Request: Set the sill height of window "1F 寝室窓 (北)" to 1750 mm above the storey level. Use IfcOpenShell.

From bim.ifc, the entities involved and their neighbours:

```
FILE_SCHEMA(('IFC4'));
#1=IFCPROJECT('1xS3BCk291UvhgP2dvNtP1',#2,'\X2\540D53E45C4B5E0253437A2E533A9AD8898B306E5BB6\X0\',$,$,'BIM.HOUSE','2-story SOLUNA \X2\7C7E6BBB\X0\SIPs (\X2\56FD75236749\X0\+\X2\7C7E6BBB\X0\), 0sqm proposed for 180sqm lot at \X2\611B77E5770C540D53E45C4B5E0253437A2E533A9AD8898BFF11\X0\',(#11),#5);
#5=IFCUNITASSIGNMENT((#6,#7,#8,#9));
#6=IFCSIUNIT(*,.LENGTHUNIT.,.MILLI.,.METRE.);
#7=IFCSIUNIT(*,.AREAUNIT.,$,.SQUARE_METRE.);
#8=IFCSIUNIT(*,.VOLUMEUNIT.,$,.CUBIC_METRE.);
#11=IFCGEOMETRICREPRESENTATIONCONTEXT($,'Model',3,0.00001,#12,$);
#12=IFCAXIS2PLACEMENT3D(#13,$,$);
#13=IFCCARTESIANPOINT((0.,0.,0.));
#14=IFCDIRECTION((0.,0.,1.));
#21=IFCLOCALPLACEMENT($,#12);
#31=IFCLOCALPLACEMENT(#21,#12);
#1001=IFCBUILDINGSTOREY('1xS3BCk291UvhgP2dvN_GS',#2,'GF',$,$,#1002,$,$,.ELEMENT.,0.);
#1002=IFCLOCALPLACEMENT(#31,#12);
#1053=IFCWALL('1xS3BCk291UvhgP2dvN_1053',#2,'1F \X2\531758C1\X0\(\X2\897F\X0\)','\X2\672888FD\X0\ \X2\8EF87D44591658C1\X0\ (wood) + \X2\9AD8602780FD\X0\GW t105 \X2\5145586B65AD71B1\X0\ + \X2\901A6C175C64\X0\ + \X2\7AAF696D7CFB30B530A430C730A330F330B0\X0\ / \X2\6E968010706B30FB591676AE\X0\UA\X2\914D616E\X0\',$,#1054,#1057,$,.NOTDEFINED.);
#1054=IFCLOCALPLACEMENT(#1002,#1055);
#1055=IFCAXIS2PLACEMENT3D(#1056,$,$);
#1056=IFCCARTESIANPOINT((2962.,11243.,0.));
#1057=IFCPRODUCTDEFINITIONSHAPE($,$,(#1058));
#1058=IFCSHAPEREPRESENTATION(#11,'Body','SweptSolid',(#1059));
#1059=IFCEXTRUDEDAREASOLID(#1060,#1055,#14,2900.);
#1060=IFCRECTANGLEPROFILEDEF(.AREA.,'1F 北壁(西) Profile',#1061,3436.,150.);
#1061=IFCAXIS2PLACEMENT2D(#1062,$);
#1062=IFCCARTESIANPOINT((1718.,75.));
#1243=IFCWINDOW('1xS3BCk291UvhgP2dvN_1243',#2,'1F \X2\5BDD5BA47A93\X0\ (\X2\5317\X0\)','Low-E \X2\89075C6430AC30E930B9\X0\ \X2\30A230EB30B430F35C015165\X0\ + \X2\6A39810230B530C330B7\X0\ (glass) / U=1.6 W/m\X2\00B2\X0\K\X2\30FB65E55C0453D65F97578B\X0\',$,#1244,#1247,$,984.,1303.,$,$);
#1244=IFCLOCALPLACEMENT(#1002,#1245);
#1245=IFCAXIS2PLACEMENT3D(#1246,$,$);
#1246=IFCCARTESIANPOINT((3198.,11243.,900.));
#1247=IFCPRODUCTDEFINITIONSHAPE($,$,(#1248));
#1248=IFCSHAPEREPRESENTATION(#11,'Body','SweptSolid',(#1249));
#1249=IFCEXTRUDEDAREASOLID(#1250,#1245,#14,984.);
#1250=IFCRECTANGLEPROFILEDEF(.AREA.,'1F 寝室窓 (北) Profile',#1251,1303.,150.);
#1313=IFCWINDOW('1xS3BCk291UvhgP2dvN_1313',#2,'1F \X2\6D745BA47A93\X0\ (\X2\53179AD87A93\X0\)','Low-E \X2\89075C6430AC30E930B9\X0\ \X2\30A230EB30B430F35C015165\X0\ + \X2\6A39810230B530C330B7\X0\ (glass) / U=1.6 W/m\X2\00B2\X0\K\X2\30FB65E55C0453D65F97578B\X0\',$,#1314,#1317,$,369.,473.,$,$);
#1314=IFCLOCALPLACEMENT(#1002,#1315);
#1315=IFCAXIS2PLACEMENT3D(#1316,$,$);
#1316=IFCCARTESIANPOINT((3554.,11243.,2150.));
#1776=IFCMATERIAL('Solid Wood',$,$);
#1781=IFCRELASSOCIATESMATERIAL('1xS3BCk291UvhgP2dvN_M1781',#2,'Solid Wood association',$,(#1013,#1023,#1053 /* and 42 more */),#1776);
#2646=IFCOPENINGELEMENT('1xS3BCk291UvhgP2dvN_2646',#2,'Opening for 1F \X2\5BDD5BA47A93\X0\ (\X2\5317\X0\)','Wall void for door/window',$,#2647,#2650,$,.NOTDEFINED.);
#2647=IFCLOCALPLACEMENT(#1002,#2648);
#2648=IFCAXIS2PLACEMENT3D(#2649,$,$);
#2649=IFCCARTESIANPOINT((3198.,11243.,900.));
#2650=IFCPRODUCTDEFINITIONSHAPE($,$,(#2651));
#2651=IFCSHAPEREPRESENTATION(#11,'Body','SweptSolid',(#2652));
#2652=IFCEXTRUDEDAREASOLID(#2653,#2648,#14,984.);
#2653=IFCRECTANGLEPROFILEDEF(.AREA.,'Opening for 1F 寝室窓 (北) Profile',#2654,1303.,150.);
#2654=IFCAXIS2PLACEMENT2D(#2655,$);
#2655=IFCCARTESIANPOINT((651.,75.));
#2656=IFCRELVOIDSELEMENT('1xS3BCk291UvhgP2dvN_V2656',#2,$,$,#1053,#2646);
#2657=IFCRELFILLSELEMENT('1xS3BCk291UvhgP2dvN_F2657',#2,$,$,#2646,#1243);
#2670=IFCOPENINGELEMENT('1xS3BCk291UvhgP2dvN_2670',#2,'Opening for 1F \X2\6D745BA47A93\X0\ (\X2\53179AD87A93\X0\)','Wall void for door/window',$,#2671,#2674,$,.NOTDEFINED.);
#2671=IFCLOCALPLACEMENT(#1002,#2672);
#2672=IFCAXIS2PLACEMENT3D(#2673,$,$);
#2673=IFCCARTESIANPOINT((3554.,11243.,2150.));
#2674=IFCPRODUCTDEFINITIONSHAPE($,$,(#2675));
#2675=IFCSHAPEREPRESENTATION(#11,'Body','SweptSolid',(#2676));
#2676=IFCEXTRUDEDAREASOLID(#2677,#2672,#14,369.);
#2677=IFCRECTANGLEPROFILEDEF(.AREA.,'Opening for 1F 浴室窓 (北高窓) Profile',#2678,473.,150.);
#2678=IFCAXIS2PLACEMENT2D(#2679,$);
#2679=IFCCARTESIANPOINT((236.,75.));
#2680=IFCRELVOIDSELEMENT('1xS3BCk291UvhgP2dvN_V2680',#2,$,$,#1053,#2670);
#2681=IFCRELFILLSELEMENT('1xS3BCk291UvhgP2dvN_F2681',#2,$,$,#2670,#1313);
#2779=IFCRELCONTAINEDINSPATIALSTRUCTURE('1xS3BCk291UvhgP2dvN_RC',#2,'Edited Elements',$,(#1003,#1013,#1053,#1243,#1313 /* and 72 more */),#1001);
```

```python
import numpy as np
import ifcopenshell
import ifcopenshell.api.geometry
import ifcopenshell.geom
import ifcopenshell.util.element
import ifcopenshell.util.placement
import ifcopenshell.util.shape
import ifcopenshell.util.unit

model = ifcopenshell.open("bim.ifc")
unit_scale = ifcopenshell.util.unit.calculate_unit_scale(model)

window = model.by_guid("1xS3BCk291UvhgP2dvN_1243")
opening = window.FillsVoids[0].RelatingOpeningElement
storey = ifcopenshell.util.element.get_container(window, ifc_class="IfcBuildingStorey")
level = ifcopenshell.util.placement.get_local_placement(storey.ObjectPlacement)[2, 3]

# The opening's origin need not be at the sill, so measure its lowest point.
shape = ifcopenshell.geom.create_shape(ifcopenshell.geom.settings(), opening)
bottom = ifcopenshell.util.shape.get_shape_bottom_elevation(shape, shape.geometry) / unit_scale
dz = level + 1.75 / unit_scale - bottom

shift = np.array([0.0, 0.0, dz])
# The window is not placed relative to its opening, so move both.
for product in (opening, window):
    matrix = ifcopenshell.util.placement.get_local_placement(product.ObjectPlacement)
    matrix[:3, 3] += shift
    ifcopenshell.api.geometry.edit_object_placement(model, product=product, matrix=matrix, is_si=False)

print(f"moved by {dz * unit_scale:+.3f} m")

model.write("bim_v2.ifc")
```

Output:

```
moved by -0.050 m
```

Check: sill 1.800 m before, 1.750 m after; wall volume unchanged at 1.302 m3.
